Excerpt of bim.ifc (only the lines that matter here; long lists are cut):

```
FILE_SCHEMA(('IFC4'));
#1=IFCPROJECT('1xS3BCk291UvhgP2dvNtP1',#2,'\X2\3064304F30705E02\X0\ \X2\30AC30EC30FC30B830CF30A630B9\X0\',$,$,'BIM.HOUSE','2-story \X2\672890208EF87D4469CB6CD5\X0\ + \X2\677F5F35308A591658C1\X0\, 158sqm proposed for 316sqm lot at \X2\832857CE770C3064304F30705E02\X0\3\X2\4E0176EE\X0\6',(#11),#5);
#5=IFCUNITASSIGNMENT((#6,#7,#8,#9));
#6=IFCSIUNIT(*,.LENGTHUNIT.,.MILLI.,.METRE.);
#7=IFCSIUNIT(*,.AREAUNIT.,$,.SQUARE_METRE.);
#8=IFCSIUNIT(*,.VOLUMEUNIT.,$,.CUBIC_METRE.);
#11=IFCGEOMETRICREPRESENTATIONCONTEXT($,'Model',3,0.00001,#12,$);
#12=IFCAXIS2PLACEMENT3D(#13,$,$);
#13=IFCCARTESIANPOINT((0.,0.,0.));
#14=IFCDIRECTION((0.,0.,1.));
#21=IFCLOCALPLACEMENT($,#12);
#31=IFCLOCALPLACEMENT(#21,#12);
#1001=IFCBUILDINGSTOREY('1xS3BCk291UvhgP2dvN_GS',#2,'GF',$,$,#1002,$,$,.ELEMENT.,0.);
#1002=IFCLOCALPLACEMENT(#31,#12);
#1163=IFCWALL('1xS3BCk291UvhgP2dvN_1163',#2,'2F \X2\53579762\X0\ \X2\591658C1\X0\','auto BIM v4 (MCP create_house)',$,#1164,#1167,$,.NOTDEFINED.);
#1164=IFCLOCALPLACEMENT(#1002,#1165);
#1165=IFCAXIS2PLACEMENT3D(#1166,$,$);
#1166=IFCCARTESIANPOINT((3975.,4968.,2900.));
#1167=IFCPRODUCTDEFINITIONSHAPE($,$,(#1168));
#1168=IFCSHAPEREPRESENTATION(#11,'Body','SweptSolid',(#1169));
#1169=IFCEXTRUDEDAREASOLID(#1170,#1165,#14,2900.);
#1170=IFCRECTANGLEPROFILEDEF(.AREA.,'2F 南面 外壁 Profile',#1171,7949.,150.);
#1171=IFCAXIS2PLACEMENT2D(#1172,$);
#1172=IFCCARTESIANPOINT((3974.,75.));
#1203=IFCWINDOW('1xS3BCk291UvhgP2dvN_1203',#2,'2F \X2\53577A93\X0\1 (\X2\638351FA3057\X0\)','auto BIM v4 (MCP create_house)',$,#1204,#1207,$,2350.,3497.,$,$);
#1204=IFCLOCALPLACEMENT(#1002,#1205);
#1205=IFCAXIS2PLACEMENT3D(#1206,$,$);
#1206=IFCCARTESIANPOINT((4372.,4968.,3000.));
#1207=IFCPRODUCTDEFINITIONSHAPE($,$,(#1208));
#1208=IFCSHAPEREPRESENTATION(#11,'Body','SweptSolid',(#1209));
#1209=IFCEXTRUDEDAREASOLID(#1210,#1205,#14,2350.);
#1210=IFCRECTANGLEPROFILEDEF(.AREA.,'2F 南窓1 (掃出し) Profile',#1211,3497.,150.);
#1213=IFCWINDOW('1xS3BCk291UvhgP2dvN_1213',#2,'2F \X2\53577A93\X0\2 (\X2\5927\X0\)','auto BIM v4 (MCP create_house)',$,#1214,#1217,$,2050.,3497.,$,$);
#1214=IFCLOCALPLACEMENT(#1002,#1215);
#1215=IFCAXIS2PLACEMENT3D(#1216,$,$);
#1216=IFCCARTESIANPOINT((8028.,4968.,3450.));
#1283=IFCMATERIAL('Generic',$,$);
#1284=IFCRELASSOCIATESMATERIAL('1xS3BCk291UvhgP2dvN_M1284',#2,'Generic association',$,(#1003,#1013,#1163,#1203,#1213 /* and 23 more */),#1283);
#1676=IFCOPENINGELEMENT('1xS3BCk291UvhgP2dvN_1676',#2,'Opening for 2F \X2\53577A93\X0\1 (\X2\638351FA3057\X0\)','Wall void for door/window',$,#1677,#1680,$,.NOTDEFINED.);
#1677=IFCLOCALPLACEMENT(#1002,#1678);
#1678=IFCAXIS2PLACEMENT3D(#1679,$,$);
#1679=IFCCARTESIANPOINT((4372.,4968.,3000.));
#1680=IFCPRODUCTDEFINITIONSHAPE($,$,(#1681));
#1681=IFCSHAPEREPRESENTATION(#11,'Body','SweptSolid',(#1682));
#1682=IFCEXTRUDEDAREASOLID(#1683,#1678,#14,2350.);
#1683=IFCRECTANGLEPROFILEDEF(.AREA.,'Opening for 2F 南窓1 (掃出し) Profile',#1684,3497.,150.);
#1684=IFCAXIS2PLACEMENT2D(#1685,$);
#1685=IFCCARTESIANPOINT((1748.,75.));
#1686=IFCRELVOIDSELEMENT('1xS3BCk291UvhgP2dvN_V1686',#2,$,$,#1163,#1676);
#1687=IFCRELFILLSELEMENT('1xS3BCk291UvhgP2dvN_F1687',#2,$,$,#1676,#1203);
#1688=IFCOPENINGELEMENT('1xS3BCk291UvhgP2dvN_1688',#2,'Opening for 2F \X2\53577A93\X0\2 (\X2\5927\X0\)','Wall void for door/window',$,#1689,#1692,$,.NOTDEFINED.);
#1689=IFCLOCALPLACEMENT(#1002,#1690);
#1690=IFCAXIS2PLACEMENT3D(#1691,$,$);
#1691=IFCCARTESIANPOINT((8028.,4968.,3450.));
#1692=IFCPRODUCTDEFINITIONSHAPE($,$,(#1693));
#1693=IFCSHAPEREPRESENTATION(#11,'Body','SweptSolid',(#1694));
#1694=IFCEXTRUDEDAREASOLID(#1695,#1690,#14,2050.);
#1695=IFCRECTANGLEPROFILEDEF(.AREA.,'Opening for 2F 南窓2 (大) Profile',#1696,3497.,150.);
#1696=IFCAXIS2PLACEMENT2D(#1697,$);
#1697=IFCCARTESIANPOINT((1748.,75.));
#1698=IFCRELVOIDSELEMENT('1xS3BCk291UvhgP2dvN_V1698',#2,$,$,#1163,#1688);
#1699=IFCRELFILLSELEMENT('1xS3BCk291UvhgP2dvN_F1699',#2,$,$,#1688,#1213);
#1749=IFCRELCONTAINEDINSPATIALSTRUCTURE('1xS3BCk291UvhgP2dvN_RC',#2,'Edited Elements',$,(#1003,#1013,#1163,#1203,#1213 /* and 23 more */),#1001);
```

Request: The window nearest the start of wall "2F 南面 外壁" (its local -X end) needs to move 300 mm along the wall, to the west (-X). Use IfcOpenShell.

```python
import ifcopenshell
import ifcopenshell.api.geometry
import ifcopenshell.util.placement

model = ifcopenshell.open("bim.ifc")

window = model.by_id(1203)
opening = window.FillsVoids[0].RelatingOpeningElement
wall = opening.VoidsElements[0].RelatingBuildingElement

wall_matrix = ifcopenshell.util.placement.get_local_placement(wall.ObjectPlacement)
shift = wall_matrix[:3, 0] * -300.0
before = ifcopenshell.util.placement.get_local_placement(window.ObjectPlacement)[:3, 3].copy()

# The window is not placed relative to its opening, so move both.
for product in (opening, window):
    matrix = ifcopenshell.util.placement.get_local_placement(product.ObjectPlacement)
    matrix[:3, 3] += shift
    ifcopenshell.api.geometry.edit_object_placement(model, product=product, matrix=matrix, is_si=False)

after = ifcopenshell.util.placement.get_local_placement(window.ObjectPlacement)[:3, 3]
print("window moved by", (after - before).round(3) + 0.0)

model.write("bim_edited.ifc")
```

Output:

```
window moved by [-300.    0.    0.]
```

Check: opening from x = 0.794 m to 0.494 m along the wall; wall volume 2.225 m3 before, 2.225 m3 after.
